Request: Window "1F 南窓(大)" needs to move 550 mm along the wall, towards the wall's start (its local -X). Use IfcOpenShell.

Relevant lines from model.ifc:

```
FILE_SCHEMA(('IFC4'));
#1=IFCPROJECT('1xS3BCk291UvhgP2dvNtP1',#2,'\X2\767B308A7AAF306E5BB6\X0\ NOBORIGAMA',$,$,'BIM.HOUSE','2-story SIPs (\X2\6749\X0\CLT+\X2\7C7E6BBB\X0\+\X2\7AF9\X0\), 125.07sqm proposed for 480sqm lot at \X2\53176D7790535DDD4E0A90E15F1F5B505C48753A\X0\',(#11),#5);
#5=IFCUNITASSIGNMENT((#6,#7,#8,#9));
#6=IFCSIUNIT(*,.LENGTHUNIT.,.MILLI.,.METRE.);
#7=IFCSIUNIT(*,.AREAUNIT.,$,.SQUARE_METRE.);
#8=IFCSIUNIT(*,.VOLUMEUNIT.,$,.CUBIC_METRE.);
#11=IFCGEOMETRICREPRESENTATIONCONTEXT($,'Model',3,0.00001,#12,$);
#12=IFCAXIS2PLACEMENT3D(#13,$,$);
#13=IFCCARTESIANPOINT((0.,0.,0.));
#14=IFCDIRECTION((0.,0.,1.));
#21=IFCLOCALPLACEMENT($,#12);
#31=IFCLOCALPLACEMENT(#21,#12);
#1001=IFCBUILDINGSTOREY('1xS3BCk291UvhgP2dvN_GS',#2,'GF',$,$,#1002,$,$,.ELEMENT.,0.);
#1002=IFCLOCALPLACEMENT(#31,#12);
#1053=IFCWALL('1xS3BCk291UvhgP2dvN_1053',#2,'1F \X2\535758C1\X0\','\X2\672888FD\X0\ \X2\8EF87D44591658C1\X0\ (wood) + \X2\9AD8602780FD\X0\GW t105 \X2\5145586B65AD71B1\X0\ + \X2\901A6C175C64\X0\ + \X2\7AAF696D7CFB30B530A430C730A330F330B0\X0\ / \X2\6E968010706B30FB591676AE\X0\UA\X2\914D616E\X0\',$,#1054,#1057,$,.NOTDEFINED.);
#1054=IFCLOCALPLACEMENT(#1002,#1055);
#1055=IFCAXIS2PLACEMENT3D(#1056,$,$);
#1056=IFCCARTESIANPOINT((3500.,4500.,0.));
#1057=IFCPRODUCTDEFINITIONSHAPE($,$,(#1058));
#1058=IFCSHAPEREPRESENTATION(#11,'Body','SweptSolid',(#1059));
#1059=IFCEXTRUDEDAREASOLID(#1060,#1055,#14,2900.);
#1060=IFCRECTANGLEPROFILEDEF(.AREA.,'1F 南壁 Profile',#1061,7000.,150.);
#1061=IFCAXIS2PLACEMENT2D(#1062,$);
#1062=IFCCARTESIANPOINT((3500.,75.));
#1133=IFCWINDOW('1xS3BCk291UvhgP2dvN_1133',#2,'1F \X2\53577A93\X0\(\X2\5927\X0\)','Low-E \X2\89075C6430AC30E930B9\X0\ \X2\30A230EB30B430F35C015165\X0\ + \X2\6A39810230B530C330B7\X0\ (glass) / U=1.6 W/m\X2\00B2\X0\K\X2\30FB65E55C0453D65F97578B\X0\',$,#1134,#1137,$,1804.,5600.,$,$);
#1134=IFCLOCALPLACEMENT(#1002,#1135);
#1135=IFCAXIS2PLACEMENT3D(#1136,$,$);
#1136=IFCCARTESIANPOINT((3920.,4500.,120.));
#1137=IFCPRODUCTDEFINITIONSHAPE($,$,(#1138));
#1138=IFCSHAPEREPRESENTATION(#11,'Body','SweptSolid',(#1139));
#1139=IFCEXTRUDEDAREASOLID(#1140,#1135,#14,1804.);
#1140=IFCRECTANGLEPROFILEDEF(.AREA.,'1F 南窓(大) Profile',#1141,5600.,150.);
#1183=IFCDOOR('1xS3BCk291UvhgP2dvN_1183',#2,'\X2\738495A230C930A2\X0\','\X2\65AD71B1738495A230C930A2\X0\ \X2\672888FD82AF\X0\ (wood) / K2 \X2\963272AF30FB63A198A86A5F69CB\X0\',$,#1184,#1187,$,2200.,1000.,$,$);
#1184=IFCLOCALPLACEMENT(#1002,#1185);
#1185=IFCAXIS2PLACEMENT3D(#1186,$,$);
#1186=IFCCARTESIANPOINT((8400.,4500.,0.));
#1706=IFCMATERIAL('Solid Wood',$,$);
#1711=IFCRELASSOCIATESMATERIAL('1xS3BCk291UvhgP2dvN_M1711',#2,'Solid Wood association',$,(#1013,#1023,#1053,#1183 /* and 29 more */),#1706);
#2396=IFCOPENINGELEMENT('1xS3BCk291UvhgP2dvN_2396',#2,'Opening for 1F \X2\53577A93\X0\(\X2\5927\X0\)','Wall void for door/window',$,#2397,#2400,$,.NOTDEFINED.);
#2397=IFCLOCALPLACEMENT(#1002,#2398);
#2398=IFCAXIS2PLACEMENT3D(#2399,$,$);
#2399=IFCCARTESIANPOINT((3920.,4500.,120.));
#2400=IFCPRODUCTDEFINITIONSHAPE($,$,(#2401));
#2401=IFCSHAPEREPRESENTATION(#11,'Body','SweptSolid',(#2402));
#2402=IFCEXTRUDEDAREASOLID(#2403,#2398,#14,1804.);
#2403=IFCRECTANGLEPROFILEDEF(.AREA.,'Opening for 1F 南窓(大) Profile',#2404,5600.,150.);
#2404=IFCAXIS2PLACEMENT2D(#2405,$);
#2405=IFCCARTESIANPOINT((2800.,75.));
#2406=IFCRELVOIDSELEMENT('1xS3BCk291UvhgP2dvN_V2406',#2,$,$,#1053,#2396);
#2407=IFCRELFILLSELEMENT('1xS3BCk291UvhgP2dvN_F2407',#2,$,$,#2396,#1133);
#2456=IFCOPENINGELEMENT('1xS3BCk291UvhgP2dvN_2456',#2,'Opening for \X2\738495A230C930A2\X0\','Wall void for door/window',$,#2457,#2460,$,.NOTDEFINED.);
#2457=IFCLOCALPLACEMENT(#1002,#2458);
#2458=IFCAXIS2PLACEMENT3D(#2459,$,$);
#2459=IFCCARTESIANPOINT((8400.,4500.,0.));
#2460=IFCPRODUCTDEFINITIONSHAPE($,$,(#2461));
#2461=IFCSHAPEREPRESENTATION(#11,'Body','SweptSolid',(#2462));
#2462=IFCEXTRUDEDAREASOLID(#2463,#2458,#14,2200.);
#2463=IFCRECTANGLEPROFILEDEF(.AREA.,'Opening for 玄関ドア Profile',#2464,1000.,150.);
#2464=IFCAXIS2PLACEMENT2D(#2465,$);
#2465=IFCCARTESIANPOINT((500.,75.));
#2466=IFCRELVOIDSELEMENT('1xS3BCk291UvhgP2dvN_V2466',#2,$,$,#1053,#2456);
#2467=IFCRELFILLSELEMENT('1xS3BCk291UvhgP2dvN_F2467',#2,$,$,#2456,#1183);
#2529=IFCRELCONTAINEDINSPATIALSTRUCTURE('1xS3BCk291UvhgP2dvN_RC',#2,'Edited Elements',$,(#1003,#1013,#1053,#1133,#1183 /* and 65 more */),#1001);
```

```python
import ifcopenshell
import ifcopenshell.api.geometry
import ifcopenshell.util.placement
import ifcopenshell.util.unit

model = ifcopenshell.open("model.ifc")
unit_scale = ifcopenshell.util.unit.calculate_unit_scale(model)

window = model.by_guid("1xS3BCk291UvhgP2dvN_1133")
opening = window.FillsVoids[0].RelatingOpeningElement
wall = opening.VoidsElements[0].RelatingBuildingElement

wall_matrix = ifcopenshell.util.placement.get_local_placement(wall.ObjectPlacement)
shift = wall_matrix[:3, 0] * -0.55 / unit_scale
before = ifcopenshell.util.placement.get_local_placement(window.ObjectPlacement)[:3, 3].copy()

# The window is not placed relative to its opening, so move both.
for product in (opening, window):
    matrix = ifcopenshell.util.placement.get_local_placement(product.ObjectPlacement)
    matrix[:3, 3] += shift
    ifcopenshell.api.geometry.edit_object_placement(model, product=product, matrix=matrix, is_si=False)

after = ifcopenshell.util.placement.get_local_placement(window.ObjectPlacement)[:3, 3]
print("window moved by", (after - before).round(3) + 0.0)

model.write("model-out.ifc")
```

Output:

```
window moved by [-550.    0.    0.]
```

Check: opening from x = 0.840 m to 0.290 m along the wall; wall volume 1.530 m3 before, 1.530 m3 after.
